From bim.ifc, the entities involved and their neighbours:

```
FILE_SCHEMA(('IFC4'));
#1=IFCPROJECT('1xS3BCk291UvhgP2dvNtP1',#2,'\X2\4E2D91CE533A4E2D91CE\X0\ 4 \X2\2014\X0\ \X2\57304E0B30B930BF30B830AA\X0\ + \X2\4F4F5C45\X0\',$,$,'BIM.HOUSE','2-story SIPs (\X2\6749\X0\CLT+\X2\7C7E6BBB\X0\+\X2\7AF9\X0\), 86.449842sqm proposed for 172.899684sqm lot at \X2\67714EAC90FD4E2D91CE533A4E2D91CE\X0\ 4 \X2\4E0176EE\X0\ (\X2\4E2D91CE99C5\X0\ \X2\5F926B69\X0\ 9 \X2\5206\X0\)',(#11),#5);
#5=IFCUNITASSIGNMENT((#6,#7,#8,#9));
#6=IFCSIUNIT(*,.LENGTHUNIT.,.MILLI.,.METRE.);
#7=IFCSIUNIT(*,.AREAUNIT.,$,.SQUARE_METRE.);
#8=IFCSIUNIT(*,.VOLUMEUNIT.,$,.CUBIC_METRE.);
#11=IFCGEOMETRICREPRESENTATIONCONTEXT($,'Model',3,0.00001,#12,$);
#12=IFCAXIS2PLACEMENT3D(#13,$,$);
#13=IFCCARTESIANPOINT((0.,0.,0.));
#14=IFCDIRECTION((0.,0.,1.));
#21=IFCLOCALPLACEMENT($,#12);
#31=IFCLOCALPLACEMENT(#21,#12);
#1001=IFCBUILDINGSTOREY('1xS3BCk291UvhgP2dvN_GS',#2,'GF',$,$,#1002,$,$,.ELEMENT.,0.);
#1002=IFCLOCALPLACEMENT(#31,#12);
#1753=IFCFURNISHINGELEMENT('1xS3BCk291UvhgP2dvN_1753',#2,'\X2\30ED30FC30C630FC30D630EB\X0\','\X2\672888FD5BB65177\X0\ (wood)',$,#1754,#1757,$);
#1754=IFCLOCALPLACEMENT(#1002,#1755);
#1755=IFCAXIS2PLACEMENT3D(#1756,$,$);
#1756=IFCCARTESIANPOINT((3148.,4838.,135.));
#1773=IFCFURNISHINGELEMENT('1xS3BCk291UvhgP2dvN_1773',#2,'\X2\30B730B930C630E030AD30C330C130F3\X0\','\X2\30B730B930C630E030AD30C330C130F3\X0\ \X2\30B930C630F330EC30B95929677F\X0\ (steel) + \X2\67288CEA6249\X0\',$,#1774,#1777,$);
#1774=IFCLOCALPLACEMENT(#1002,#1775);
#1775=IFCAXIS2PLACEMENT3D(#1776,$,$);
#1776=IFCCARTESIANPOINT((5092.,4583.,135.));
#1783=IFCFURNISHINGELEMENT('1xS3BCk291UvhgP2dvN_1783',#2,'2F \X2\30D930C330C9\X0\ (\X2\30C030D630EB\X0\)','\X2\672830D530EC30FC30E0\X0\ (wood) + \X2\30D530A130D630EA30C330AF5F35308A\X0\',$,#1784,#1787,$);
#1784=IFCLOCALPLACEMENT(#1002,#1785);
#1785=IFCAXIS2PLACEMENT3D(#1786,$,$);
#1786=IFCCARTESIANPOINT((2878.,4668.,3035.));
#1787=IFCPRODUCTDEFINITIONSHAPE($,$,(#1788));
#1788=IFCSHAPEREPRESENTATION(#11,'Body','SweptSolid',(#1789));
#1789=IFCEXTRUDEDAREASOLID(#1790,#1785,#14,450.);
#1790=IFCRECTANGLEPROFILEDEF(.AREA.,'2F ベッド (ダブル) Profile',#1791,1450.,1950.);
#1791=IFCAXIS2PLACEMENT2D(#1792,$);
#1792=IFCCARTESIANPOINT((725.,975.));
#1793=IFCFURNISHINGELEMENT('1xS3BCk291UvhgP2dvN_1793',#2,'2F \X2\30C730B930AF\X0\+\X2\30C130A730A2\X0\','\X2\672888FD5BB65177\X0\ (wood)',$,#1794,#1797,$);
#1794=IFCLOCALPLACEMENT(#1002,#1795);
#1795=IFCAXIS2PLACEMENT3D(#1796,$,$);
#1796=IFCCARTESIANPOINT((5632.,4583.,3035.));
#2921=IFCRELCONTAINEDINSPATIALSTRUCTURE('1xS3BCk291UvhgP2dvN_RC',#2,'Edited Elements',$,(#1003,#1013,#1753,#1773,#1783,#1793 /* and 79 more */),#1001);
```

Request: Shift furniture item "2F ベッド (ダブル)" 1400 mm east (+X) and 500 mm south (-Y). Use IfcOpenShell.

```python
import ifcopenshell
import ifcopenshell.api.geometry
import ifcopenshell.util.placement
import ifcopenshell.util.unit

model = ifcopenshell.open("bim.ifc")
unit_scale = ifcopenshell.util.unit.calculate_unit_scale(model)

item = model.by_guid("1xS3BCk291UvhgP2dvN_1783")
matrix = ifcopenshell.util.placement.get_local_placement(item.ObjectPlacement)
matrix[0, 3] += 1.4 / unit_scale
matrix[1, 3] -= 0.5 / unit_scale
ifcopenshell.api.geometry.edit_object_placement(model, product=item, matrix=matrix, is_si=False)

print(ifcopenshell.util.placement.get_local_placement(item.ObjectPlacement).round(3) + 0.0)

model.write("bim_updated.ifc")
```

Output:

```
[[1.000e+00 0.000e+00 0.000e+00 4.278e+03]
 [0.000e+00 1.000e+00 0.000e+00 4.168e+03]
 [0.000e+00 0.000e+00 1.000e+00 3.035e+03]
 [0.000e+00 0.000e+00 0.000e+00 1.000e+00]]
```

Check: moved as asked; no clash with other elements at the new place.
